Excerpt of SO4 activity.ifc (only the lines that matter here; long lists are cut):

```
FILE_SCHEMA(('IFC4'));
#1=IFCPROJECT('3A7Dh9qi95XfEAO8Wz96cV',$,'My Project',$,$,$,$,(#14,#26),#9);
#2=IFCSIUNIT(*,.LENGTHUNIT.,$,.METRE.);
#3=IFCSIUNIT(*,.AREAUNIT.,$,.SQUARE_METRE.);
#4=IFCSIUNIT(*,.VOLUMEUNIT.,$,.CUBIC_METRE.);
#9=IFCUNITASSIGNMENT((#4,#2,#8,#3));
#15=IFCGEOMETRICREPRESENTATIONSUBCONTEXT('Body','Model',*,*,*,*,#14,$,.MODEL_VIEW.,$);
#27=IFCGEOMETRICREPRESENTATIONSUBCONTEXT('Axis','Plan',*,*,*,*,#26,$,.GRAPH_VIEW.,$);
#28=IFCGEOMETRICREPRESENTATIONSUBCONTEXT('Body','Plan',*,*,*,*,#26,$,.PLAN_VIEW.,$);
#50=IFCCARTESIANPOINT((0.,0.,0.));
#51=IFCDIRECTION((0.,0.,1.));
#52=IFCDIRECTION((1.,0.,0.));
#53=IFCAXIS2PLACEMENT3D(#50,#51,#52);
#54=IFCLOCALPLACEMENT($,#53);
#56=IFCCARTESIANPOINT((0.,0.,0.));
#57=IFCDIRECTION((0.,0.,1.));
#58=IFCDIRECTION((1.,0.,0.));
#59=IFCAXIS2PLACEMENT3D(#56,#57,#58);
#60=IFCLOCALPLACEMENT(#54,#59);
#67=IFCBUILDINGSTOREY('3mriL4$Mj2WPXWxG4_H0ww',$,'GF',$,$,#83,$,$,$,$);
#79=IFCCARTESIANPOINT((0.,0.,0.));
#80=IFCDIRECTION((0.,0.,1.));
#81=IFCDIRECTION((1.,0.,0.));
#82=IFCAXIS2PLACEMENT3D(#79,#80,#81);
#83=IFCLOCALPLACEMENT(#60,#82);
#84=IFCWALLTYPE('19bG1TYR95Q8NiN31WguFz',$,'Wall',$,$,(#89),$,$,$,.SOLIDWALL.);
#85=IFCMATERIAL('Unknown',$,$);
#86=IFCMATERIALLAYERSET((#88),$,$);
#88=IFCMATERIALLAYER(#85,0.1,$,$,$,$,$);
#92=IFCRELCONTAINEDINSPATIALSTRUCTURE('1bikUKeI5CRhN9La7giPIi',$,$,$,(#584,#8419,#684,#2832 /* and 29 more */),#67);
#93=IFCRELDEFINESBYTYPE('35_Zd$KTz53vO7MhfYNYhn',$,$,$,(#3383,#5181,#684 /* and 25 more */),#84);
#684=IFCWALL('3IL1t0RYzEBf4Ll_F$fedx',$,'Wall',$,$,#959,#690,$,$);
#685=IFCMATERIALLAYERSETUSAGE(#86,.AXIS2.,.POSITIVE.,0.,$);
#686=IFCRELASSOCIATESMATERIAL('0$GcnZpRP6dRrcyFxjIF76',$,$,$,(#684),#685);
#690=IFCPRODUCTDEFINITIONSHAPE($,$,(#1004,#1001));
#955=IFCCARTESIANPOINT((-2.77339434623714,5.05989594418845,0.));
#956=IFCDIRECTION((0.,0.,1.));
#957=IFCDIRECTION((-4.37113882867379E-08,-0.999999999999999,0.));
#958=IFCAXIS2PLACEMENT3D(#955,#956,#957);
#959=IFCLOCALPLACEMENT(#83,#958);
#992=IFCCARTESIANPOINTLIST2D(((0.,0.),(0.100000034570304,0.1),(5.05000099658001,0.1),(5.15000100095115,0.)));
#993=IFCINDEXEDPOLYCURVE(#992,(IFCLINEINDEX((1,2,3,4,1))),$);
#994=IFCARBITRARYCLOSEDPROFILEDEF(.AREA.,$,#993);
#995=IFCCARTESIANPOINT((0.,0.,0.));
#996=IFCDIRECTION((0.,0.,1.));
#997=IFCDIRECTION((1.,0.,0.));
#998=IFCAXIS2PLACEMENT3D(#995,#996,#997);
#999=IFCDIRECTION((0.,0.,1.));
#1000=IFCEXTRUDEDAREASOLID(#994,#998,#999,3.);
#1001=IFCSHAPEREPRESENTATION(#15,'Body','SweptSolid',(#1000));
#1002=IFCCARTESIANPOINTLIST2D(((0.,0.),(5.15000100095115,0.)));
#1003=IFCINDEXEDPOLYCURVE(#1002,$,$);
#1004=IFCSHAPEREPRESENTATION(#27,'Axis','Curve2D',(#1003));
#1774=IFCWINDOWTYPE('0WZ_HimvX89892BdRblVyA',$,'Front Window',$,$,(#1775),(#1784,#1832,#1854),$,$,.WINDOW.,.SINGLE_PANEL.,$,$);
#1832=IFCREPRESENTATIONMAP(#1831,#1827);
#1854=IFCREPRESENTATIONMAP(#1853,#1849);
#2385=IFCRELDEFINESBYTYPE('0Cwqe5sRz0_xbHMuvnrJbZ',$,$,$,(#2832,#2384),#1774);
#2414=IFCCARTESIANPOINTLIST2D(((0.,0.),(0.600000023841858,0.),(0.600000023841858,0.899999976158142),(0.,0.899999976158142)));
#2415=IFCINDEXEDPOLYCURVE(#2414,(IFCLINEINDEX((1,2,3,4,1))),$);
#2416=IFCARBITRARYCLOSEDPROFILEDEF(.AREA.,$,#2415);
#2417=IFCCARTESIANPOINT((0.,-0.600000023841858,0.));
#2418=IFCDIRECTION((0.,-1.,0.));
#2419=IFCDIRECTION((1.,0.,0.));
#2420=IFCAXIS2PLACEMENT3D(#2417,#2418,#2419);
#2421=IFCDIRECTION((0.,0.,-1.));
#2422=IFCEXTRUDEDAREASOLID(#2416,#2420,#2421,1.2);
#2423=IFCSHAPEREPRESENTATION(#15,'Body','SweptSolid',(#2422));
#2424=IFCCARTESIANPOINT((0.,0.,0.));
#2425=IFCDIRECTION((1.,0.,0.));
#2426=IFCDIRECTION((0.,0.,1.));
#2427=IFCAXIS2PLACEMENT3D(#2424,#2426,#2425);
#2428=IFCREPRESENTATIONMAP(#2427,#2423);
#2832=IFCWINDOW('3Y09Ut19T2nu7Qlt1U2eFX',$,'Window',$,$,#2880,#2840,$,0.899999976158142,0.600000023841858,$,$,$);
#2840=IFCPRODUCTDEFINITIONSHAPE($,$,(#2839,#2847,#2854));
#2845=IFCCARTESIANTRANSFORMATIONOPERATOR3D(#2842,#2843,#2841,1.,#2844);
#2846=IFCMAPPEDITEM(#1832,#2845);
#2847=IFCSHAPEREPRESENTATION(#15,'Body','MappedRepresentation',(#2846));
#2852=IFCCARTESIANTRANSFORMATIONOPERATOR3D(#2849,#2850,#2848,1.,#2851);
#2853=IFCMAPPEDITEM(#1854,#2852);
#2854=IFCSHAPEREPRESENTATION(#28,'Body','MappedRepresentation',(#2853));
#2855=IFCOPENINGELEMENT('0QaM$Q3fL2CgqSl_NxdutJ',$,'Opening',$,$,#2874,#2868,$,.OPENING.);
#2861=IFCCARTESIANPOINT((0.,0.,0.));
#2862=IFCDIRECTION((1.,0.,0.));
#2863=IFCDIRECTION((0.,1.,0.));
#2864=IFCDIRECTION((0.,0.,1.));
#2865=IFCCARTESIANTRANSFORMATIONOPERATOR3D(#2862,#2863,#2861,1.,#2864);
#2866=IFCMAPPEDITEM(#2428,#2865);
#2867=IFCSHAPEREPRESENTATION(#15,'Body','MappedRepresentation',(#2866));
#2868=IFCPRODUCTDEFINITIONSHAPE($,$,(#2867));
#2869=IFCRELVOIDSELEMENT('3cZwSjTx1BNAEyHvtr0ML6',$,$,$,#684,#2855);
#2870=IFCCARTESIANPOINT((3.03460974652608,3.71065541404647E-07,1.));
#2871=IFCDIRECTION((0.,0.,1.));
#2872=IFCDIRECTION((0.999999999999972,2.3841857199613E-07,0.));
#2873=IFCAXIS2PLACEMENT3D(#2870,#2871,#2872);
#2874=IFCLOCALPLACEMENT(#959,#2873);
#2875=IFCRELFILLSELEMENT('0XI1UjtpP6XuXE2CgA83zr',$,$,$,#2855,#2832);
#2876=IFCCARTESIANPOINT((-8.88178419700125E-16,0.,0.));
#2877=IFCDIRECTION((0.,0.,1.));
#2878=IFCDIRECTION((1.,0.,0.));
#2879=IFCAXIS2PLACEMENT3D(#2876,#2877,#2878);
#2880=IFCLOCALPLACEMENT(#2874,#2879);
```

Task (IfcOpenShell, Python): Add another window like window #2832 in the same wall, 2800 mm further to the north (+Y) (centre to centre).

```python
import ifcopenshell
import ifcopenshell.api.feature
import ifcopenshell.api.geometry
import ifcopenshell.api.root
import ifcopenshell.geom
import ifcopenshell.util.element
import ifcopenshell.util.placement
import ifcopenshell.util.shape
import ifcopenshell.util.unit

model = ifcopenshell.open("SO4 activity.ifc")
unit_scale = ifcopenshell.util.unit.calculate_unit_scale(model)
settings = ifcopenshell.geom.settings()


def volume(element):
    """Net volume in cubic metres, openings subtracted."""
    shape = ifcopenshell.geom.create_shape(settings, element)
    return ifcopenshell.util.shape.get_volume(shape.geometry)


window = model.by_id(2832)
opening = window.FillsVoids[0].RelatingOpeningElement
wall = opening.VoidsElements[0].RelatingBuildingElement
before = volume(wall)
shift = ifcopenshell.util.placement.get_local_placement(wall.ObjectPlacement)[:3, 0] * -2.8 / unit_scale

# copy_class copies the void relationship, type, container and properties, but no geometry.
new_opening = ifcopenshell.api.root.copy_class(model, product=opening)
new_opening.Representation = ifcopenshell.util.element.copy_deep(
    model, opening.Representation, exclude=["IfcGeometricRepresentationContext", "IfcRepresentationMap"]
)
new_window = ifcopenshell.api.root.copy_class(model, product=window)
new_window.Representation = ifcopenshell.util.element.copy_deep(
    model, window.Representation, exclude=["IfcGeometricRepresentationContext", "IfcRepresentationMap"]
)
ifcopenshell.api.feature.add_filling(model, opening=new_opening, element=new_window)

for old, new in ((opening, new_opening), (window, new_window)):
    matrix = ifcopenshell.util.placement.get_local_placement(old.ObjectPlacement)
    matrix[:3, 3] += shift
    ifcopenshell.api.geometry.edit_object_placement(model, product=new, matrix=matrix, is_si=False)

after = volume(wall)

print(f"wall volume {before:.3f} -> {after:.3f} m3")

model.write("SO4 activity_edited.ifc")
```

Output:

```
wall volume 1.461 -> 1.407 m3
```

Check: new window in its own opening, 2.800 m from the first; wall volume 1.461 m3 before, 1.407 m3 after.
